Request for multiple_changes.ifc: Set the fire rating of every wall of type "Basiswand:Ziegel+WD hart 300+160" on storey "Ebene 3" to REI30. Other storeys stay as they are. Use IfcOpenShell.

First a look at what the model holds.

```python
import ifcopenshell
import ifcopenshell.util.element

model = ifcopenshell.open("multiple_changes.ifc")
print(model.schema)
storey = next(s for s in model.by_type("IfcBuildingStorey") if s.Name == "Ebene 3")
walls = [e for e in ifcopenshell.util.element.get_decomposition(storey) if e.is_a("IfcWall")]
seen = {}
for e in walls:
    element_type = ifcopenshell.util.element.get_type(e)
    key = (element_type.Name if element_type != e and element_type else None, ifcopenshell.util.element.get_pset(e, "Pset_WallCommon", "FireRating"))
    seen[key] = seen.get(key, 0) + 1
for (name, value), count in sorted(seen.items(), key=str):
    print(count, "x", name, "|", value)
```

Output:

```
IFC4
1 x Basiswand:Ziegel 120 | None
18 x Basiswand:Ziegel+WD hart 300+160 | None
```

```python
import ifcopenshell
import ifcopenshell.api.pset
import ifcopenshell.util.element

model = ifcopenshell.open("multiple_changes.ifc")

storey = next(s for s in model.by_type("IfcBuildingStorey") if s.Name == "Ebene 3")
walls = [e for e in ifcopenshell.util.element.get_decomposition(storey) if e.is_a("IfcWall")]

count = 0
for e in walls:
    element_type = ifcopenshell.util.element.get_type(e)
    if element_type in (None, e) or element_type.Name != "Basiswand:Ziegel+WD hart 300+160":
        continue
    # add_pset returns the element's existing set when there is one.
    pset = ifcopenshell.api.pset.add_pset(model, product=e, name="Pset_WallCommon")
    ifcopenshell.api.pset.edit_pset(model, pset=pset, properties={"FireRating": "REI30"})
    count += 1

print(count, "walls updated")

model.write("multiple_changes_edited.ifc")
```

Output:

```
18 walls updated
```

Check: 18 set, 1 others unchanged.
